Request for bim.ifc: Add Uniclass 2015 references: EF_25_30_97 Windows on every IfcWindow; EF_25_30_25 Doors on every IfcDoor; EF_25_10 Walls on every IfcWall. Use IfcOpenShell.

First a look at what the model holds.

```python
import ifcopenshell

model = ifcopenshell.open("bim.ifc")
print(model.schema)
print("classifications:", [c.Name for c in model.by_type("IfcClassification")])
for ifc_class in ("IfcDoor", "IfcRoof", "IfcStair", "IfcWall", "IfcWindow"):
    print(ifc_class, len(model.by_type(ifc_class)))
```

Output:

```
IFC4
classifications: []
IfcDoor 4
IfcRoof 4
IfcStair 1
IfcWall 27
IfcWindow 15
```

```python
import ifcopenshell
import ifcopenshell.api.classification

model = ifcopenshell.open("bim.ifc")

system = ifcopenshell.api.classification.add_classification(model, classification="Uniclass 2015")

codes = {
    "IfcWindow": ("EF_25_30_97", "Windows"),
    "IfcDoor": ("EF_25_30_25", "Doors"),
    "IfcWall": ("EF_25_10", "Walls"),
}
for ifc_class, (code, name) in codes.items():
    products = model.by_type(ifc_class)
    ifcopenshell.api.classification.add_reference(
        model, products=products, classification=system, identification=code, name=name
    )
    print(code, len(products))

model.write("bim_edited.ifc")
```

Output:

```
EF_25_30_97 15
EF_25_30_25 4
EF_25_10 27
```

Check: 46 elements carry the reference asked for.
